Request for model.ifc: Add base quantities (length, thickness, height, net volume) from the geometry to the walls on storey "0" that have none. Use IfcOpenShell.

First a look at what the model holds.

```python
import ifcopenshell
import ifcopenshell.util.element
import ifcopenshell.util.unit

model = ifcopenshell.open("model.ifc")
print(model.schema)
for unit_type in ("LENGTHUNIT", "AREAUNIT", "VOLUMEUNIT"):
    print(unit_type, ifcopenshell.util.unit.calculate_unit_scale(model, unit_type))
storey = next(s for s in model.by_type("IfcBuildingStorey") if s.Name == "0")
walls = [e for e in ifcopenshell.util.element.get_decomposition(storey) if e.is_a("IfcWall")]
for e in sorted(walls, key=lambda e: e.id()):
    print(e.id(), e.is_a(), e.Name, list(ifcopenshell.util.element.get_psets(e, qtos_only=True)), sep=" | ")
```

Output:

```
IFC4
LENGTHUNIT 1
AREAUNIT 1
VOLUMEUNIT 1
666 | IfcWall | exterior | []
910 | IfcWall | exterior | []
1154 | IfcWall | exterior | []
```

```python
import ifcopenshell
import ifcopenshell.api.pset
import ifcopenshell.geom
import ifcopenshell.util.element
import ifcopenshell.util.shape
import ifcopenshell.util.unit

model = ifcopenshell.open("model.ifc")
unit_scale = ifcopenshell.util.unit.calculate_unit_scale(model)
volume_scale = ifcopenshell.util.unit.calculate_unit_scale(model, "VOLUMEUNIT")
settings = ifcopenshell.geom.settings()

storey = next(s for s in model.by_type("IfcBuildingStorey") if s.Name == "0")
walls = [e for e in ifcopenshell.util.element.get_decomposition(storey) if e.is_a("IfcWall")]

for e in sorted(walls, key=lambda e: e.id()):
    if ifcopenshell.util.element.get_psets(e, qtos_only=True, should_inherit=False):
        continue
    # Geometry comes back in metres, in the element's own axes.
    shape = ifcopenshell.geom.create_shape(settings, e)
    values = {
        "Length": ifcopenshell.util.shape.get_x(shape.geometry) / unit_scale,
        "Width": ifcopenshell.util.shape.get_y(shape.geometry) / unit_scale,
        "Height": ifcopenshell.util.shape.get_z(shape.geometry) / unit_scale,
        "NetVolume": ifcopenshell.util.shape.get_volume(shape.geometry) / volume_scale,
    }
    qto = ifcopenshell.api.pset.add_qto(model, product=e, name="Qto_WallBaseQuantities")
    ifcopenshell.api.pset.edit_qto(model, qto=qto, properties=values)
    print(e.id(), {k: round(v, 3) for k, v in values.items()})

model.write("model_updated.ifc")
```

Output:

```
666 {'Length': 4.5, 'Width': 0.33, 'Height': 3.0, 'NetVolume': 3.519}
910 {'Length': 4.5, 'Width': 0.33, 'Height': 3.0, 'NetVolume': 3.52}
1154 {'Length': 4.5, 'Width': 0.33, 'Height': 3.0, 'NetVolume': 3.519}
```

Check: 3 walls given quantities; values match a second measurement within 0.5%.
